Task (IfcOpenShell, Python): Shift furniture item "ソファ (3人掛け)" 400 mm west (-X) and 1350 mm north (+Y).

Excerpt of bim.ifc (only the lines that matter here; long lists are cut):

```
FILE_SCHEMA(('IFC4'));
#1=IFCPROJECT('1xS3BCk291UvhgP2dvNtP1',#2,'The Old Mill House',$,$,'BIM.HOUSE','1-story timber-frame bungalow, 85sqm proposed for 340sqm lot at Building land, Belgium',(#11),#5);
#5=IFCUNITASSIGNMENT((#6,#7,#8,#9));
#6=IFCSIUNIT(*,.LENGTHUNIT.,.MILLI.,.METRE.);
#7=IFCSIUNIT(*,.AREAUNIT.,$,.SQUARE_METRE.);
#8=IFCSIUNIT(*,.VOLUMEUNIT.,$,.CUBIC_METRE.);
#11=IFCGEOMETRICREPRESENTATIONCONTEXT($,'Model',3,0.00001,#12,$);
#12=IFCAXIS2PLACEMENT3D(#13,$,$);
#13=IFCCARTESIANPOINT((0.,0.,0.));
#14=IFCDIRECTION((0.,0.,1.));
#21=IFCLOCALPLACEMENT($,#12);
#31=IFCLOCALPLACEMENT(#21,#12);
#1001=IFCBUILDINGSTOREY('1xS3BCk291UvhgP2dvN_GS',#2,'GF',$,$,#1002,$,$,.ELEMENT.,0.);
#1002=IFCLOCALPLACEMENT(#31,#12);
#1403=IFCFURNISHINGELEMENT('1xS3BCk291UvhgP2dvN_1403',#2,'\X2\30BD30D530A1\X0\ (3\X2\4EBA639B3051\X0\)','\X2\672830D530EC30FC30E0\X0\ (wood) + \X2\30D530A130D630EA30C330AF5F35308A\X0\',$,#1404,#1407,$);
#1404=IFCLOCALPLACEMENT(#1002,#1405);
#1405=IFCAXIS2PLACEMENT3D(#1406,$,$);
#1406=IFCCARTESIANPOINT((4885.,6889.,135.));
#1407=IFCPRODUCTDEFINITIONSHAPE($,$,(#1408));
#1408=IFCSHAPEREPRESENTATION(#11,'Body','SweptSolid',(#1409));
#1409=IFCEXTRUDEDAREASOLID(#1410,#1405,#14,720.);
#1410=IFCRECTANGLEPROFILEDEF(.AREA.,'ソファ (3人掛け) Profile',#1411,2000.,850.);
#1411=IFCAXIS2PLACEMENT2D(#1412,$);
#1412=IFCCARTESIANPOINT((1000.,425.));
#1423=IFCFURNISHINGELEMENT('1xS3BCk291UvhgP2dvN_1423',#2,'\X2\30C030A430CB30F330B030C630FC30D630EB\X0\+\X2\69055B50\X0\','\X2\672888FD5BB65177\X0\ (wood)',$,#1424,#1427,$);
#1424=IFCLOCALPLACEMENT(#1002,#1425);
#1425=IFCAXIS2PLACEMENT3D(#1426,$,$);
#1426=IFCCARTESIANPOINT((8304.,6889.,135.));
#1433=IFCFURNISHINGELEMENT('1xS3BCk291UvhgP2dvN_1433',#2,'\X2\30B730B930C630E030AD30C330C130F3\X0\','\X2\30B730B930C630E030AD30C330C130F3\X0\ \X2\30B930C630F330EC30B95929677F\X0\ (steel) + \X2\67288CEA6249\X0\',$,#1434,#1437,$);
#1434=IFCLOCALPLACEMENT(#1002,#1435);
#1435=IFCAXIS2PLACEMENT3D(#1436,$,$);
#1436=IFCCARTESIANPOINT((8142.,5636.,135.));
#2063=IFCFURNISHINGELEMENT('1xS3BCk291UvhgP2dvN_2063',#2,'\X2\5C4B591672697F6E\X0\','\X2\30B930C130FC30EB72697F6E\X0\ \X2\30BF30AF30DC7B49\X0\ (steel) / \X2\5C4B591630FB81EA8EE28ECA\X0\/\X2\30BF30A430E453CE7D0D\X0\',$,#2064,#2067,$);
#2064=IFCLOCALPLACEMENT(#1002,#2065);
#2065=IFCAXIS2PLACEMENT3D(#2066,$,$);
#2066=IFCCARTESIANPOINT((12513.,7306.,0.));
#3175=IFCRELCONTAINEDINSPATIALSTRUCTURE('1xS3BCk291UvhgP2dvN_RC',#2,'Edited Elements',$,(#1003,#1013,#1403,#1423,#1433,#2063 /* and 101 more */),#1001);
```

```python
import ifcopenshell
import ifcopenshell.api.geometry
import ifcopenshell.util.placement
import ifcopenshell.util.unit

model = ifcopenshell.open("bim.ifc")
unit_scale = ifcopenshell.util.unit.calculate_unit_scale(model)

item = model.by_id(1403)
matrix = ifcopenshell.util.placement.get_local_placement(item.ObjectPlacement)
matrix[0, 3] -= 0.4 / unit_scale
matrix[1, 3] += 1.35 / unit_scale
ifcopenshell.api.geometry.edit_object_placement(model, product=item, matrix=matrix, is_si=False)

print(ifcopenshell.util.placement.get_local_placement(item.ObjectPlacement).round(3) + 0.0)

model.write("bim_rev.ifc")
```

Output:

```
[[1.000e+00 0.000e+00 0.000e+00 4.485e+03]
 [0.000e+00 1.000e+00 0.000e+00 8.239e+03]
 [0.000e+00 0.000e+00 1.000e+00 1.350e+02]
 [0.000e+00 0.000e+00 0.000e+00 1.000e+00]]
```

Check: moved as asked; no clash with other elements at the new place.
